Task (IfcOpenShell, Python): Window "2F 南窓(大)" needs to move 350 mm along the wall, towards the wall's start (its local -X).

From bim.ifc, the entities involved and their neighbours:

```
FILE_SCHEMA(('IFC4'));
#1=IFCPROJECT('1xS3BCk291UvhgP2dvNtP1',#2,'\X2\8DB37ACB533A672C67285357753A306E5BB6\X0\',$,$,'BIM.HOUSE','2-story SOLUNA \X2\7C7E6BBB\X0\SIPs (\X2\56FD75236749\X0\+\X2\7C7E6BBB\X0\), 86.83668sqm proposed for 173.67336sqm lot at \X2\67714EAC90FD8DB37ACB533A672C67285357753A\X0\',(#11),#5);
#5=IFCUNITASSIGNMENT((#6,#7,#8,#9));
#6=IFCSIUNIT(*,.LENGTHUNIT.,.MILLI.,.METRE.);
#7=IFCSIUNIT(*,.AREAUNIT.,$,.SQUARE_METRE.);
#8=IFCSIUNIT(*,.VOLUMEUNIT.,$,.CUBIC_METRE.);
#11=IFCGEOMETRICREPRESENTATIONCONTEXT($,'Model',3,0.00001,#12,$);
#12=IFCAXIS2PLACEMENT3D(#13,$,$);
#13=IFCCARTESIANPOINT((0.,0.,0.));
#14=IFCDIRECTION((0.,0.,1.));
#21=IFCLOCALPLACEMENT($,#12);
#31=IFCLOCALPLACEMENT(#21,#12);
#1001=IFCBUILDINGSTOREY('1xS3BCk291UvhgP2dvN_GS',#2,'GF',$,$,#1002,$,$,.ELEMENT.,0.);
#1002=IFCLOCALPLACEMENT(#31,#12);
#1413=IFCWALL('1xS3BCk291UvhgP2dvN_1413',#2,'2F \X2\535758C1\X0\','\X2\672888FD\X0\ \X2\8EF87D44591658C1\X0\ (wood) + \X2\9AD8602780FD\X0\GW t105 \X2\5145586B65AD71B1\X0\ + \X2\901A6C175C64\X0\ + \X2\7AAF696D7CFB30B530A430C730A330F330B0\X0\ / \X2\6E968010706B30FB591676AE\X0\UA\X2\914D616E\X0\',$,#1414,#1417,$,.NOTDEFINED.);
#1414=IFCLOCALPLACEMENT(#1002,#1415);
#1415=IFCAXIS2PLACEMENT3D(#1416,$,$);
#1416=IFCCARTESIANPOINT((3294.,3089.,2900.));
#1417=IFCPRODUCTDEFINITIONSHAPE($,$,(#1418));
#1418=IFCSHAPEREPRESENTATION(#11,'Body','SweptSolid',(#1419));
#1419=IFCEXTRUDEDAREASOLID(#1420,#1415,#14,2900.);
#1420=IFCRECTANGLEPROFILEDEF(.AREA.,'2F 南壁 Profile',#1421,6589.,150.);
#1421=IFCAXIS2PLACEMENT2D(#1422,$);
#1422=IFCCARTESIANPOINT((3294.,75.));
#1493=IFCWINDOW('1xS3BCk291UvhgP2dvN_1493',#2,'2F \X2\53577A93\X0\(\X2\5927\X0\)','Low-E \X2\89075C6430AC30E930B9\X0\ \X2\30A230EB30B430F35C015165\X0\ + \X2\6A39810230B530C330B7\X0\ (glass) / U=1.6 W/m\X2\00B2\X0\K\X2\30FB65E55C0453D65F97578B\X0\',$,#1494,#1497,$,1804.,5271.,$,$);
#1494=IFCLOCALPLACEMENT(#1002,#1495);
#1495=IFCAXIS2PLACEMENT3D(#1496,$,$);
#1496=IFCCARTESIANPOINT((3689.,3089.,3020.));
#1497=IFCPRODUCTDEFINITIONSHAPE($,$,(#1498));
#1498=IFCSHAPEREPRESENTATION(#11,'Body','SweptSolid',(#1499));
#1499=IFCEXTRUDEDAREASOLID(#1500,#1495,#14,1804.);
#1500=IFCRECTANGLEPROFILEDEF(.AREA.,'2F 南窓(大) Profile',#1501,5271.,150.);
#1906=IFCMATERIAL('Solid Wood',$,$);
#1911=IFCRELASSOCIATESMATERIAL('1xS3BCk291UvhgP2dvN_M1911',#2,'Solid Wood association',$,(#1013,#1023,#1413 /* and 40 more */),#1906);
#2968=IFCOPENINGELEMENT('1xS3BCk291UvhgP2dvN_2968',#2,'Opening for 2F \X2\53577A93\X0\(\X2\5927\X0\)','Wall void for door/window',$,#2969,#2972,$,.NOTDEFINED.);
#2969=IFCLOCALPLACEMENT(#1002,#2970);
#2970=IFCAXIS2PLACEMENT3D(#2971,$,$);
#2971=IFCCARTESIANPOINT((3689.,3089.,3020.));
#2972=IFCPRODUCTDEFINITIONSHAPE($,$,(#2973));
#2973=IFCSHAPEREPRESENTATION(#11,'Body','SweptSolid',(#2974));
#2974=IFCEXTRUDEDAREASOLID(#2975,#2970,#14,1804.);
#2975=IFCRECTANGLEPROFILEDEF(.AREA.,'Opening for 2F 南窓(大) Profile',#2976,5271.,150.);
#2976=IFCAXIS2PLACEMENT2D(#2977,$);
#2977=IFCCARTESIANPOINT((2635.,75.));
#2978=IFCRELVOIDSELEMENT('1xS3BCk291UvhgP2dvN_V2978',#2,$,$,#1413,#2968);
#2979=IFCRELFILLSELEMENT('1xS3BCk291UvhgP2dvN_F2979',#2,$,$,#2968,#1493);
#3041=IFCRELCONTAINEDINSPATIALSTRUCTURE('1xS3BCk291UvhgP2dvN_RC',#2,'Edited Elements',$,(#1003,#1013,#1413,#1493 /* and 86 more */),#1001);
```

```python
import ifcopenshell
import ifcopenshell.api.geometry
import ifcopenshell.util.placement

model = ifcopenshell.open("bim.ifc")

window = model.by_id(1493)
opening = window.FillsVoids[0].RelatingOpeningElement
wall = opening.VoidsElements[0].RelatingBuildingElement

wall_matrix = ifcopenshell.util.placement.get_local_placement(wall.ObjectPlacement)
shift = wall_matrix[:3, 0] * -350.0
before = ifcopenshell.util.placement.get_local_placement(window.ObjectPlacement)[:3, 3].copy()

# The window is not placed relative to its opening, so move both.
for product in (opening, window):
    matrix = ifcopenshell.util.placement.get_local_placement(product.ObjectPlacement)
    matrix[:3, 3] += shift
    ifcopenshell.api.geometry.edit_object_placement(model, product=product, matrix=matrix, is_si=False)

after = ifcopenshell.util.placement.get_local_placement(window.ObjectPlacement)[:3, 3]
print("window moved by", (after - before).round(3) + 0.0)

model.write("bim_edited.ifc")
```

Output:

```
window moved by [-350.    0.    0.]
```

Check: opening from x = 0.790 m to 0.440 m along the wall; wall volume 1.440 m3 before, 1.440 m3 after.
